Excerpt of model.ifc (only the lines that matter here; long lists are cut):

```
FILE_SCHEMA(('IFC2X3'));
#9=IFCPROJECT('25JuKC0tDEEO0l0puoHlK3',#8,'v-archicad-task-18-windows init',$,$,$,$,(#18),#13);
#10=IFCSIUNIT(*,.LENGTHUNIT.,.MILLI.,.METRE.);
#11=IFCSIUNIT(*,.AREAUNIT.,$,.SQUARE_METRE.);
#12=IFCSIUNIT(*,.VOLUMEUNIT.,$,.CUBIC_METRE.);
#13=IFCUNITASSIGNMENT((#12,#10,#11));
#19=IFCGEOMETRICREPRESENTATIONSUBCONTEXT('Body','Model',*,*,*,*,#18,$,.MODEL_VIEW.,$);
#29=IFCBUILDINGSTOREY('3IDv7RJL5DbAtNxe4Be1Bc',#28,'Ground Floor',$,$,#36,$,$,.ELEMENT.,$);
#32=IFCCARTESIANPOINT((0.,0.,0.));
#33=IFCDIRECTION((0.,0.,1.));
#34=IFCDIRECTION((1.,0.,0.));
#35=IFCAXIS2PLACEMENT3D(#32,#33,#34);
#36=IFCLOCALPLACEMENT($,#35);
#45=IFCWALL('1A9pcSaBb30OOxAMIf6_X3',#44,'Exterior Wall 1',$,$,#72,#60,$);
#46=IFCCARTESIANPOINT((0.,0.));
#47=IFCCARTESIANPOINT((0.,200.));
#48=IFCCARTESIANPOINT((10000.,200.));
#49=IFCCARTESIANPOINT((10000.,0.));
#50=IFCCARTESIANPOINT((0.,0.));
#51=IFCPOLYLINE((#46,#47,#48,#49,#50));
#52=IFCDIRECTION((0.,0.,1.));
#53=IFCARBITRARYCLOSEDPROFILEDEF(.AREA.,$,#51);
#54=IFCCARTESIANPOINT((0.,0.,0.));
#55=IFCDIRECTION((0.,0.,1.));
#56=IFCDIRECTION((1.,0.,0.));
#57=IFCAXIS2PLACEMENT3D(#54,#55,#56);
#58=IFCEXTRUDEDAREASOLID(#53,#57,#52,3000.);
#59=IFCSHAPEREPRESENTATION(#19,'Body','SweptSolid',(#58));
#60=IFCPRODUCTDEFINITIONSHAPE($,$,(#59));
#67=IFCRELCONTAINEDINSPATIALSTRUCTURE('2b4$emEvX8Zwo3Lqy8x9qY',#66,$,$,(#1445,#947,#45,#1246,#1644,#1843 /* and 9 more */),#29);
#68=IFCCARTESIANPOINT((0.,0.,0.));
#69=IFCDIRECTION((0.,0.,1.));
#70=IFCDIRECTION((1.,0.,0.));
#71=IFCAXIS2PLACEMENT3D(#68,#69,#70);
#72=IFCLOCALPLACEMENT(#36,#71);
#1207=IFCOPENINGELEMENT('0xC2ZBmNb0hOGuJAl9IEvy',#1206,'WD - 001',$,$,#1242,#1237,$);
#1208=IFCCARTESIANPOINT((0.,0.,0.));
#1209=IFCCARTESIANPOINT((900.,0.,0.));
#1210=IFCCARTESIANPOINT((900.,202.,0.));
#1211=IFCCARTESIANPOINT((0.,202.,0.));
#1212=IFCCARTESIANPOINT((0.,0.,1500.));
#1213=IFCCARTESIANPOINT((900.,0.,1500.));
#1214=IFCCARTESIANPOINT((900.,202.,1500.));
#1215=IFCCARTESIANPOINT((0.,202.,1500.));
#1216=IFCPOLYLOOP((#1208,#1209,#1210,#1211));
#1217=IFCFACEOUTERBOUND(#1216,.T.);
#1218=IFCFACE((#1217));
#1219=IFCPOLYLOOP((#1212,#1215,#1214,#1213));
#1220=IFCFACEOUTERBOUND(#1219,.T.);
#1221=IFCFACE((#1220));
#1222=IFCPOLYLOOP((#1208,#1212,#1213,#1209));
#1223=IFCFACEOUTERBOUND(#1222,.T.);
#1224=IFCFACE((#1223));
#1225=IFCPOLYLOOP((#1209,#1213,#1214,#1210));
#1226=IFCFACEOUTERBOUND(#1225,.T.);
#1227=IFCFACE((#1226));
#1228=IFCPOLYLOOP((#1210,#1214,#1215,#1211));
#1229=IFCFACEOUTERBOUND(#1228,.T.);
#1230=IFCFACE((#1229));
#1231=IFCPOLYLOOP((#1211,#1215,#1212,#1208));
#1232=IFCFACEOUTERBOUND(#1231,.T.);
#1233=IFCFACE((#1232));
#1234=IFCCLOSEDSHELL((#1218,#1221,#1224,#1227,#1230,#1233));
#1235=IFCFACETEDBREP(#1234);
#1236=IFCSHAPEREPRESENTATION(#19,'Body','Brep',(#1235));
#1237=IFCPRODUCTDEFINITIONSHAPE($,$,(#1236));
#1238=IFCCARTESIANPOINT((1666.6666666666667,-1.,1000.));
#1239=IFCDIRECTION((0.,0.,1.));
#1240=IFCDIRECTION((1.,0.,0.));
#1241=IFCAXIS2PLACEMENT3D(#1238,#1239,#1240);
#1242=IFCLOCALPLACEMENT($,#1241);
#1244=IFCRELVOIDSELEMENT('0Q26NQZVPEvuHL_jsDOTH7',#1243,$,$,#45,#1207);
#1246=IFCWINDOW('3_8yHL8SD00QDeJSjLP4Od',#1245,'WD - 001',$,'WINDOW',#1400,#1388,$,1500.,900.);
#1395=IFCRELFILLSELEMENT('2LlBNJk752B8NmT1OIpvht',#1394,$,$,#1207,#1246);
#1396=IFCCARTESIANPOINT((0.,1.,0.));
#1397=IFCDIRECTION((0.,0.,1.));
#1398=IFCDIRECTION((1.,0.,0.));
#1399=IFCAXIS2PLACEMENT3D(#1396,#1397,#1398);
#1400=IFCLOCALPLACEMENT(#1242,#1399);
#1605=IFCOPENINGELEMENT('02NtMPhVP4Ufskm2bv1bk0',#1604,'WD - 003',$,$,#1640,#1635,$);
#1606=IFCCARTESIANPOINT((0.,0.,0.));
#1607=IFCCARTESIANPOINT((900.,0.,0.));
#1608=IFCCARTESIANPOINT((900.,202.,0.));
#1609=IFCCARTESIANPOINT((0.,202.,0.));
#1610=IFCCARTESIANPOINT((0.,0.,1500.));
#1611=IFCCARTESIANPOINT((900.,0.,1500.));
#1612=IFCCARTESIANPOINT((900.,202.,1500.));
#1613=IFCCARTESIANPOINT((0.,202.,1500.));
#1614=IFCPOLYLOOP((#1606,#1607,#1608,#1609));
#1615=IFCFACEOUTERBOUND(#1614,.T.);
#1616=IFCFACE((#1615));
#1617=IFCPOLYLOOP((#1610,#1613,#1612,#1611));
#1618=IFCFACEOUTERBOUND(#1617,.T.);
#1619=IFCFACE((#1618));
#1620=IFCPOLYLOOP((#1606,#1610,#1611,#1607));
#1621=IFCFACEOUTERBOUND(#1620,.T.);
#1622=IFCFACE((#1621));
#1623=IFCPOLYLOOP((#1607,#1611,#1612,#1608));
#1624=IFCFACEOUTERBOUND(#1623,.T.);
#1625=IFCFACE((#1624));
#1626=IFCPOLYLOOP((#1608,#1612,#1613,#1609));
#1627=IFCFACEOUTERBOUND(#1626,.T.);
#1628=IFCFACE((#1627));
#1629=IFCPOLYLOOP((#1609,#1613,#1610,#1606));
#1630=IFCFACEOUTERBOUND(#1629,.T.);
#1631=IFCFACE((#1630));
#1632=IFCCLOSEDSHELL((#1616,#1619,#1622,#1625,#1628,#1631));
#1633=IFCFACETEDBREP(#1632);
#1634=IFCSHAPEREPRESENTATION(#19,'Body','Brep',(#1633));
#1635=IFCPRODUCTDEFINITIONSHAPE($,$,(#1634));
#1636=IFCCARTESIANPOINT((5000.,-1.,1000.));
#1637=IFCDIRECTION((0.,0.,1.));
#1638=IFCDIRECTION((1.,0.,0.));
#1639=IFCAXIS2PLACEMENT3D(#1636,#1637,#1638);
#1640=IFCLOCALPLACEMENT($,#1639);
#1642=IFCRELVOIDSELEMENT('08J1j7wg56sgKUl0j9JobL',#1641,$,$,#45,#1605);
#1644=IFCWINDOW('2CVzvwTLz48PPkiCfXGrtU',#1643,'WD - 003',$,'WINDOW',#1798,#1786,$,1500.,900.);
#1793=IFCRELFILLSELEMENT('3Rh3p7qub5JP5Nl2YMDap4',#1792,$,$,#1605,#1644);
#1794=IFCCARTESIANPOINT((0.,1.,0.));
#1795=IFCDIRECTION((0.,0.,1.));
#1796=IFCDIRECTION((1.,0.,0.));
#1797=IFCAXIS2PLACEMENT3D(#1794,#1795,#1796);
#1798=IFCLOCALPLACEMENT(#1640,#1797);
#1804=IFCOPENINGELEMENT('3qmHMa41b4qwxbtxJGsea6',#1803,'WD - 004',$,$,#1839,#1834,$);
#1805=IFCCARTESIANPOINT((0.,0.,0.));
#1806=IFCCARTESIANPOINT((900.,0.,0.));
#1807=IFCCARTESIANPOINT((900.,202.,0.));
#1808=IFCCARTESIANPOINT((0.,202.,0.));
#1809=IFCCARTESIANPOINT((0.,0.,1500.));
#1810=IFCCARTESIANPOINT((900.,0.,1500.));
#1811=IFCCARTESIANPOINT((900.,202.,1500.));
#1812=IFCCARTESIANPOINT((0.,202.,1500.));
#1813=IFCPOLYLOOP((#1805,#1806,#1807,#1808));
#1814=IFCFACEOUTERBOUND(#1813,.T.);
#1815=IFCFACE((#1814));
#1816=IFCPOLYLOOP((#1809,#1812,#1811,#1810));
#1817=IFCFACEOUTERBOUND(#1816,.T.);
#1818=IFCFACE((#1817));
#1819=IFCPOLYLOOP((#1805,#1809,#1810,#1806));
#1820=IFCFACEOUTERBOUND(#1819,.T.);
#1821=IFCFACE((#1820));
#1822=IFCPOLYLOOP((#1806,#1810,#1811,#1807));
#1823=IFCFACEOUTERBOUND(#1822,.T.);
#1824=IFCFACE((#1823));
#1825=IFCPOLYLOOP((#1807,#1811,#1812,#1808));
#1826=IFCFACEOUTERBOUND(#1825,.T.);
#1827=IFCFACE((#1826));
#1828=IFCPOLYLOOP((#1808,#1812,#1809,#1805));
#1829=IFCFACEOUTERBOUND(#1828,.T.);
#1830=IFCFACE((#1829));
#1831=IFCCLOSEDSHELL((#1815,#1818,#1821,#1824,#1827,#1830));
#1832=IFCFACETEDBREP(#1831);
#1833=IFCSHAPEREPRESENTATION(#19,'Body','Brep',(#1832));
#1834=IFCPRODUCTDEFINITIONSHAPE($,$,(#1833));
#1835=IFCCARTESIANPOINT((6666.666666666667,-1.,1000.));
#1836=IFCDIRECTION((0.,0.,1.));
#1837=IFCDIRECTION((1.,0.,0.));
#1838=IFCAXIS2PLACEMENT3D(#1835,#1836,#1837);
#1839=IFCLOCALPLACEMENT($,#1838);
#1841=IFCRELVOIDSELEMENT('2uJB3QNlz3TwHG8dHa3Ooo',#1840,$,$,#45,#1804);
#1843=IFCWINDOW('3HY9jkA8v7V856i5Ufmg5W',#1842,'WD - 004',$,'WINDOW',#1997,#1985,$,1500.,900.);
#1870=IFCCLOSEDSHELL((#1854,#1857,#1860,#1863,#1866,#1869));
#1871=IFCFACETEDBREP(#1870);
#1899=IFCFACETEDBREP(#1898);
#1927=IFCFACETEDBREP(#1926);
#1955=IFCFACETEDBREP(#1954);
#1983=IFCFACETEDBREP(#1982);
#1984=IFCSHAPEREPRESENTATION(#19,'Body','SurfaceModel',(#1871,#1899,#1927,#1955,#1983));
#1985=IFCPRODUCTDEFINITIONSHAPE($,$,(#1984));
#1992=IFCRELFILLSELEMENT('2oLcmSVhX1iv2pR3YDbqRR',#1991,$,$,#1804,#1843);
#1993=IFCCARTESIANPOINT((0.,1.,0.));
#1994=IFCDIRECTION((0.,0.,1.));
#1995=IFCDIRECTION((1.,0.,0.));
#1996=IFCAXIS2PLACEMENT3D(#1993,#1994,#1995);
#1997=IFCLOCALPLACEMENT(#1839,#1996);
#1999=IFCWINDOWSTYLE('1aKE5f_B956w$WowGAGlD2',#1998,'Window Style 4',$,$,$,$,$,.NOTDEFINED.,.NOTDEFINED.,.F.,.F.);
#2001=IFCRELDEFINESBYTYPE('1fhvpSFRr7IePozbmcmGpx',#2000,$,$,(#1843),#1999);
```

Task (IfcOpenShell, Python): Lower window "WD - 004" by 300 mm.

```python
import numpy as np
import ifcopenshell
import ifcopenshell.api.geometry
import ifcopenshell.util.placement
import ifcopenshell.util.unit

model = ifcopenshell.open("model.ifc")
unit_scale = ifcopenshell.util.unit.calculate_unit_scale(model)

window = model.by_id(1843)
opening = window.FillsVoids[0].RelatingOpeningElement
dz = -0.3 / unit_scale

shift = np.array([0.0, 0.0, dz])
# The window is placed relative to its opening, so it follows when the opening moves.
matrix = ifcopenshell.util.placement.get_local_placement(opening.ObjectPlacement)
matrix[:3, 3] += shift
ifcopenshell.api.geometry.edit_object_placement(
    model, product=opening, matrix=matrix, is_si=False, should_transform_children=True
)

print(f"moved by {dz * unit_scale:+.3f} m")

model.write("model_updated.ifc")
```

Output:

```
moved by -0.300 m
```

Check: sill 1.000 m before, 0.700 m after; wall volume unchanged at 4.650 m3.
